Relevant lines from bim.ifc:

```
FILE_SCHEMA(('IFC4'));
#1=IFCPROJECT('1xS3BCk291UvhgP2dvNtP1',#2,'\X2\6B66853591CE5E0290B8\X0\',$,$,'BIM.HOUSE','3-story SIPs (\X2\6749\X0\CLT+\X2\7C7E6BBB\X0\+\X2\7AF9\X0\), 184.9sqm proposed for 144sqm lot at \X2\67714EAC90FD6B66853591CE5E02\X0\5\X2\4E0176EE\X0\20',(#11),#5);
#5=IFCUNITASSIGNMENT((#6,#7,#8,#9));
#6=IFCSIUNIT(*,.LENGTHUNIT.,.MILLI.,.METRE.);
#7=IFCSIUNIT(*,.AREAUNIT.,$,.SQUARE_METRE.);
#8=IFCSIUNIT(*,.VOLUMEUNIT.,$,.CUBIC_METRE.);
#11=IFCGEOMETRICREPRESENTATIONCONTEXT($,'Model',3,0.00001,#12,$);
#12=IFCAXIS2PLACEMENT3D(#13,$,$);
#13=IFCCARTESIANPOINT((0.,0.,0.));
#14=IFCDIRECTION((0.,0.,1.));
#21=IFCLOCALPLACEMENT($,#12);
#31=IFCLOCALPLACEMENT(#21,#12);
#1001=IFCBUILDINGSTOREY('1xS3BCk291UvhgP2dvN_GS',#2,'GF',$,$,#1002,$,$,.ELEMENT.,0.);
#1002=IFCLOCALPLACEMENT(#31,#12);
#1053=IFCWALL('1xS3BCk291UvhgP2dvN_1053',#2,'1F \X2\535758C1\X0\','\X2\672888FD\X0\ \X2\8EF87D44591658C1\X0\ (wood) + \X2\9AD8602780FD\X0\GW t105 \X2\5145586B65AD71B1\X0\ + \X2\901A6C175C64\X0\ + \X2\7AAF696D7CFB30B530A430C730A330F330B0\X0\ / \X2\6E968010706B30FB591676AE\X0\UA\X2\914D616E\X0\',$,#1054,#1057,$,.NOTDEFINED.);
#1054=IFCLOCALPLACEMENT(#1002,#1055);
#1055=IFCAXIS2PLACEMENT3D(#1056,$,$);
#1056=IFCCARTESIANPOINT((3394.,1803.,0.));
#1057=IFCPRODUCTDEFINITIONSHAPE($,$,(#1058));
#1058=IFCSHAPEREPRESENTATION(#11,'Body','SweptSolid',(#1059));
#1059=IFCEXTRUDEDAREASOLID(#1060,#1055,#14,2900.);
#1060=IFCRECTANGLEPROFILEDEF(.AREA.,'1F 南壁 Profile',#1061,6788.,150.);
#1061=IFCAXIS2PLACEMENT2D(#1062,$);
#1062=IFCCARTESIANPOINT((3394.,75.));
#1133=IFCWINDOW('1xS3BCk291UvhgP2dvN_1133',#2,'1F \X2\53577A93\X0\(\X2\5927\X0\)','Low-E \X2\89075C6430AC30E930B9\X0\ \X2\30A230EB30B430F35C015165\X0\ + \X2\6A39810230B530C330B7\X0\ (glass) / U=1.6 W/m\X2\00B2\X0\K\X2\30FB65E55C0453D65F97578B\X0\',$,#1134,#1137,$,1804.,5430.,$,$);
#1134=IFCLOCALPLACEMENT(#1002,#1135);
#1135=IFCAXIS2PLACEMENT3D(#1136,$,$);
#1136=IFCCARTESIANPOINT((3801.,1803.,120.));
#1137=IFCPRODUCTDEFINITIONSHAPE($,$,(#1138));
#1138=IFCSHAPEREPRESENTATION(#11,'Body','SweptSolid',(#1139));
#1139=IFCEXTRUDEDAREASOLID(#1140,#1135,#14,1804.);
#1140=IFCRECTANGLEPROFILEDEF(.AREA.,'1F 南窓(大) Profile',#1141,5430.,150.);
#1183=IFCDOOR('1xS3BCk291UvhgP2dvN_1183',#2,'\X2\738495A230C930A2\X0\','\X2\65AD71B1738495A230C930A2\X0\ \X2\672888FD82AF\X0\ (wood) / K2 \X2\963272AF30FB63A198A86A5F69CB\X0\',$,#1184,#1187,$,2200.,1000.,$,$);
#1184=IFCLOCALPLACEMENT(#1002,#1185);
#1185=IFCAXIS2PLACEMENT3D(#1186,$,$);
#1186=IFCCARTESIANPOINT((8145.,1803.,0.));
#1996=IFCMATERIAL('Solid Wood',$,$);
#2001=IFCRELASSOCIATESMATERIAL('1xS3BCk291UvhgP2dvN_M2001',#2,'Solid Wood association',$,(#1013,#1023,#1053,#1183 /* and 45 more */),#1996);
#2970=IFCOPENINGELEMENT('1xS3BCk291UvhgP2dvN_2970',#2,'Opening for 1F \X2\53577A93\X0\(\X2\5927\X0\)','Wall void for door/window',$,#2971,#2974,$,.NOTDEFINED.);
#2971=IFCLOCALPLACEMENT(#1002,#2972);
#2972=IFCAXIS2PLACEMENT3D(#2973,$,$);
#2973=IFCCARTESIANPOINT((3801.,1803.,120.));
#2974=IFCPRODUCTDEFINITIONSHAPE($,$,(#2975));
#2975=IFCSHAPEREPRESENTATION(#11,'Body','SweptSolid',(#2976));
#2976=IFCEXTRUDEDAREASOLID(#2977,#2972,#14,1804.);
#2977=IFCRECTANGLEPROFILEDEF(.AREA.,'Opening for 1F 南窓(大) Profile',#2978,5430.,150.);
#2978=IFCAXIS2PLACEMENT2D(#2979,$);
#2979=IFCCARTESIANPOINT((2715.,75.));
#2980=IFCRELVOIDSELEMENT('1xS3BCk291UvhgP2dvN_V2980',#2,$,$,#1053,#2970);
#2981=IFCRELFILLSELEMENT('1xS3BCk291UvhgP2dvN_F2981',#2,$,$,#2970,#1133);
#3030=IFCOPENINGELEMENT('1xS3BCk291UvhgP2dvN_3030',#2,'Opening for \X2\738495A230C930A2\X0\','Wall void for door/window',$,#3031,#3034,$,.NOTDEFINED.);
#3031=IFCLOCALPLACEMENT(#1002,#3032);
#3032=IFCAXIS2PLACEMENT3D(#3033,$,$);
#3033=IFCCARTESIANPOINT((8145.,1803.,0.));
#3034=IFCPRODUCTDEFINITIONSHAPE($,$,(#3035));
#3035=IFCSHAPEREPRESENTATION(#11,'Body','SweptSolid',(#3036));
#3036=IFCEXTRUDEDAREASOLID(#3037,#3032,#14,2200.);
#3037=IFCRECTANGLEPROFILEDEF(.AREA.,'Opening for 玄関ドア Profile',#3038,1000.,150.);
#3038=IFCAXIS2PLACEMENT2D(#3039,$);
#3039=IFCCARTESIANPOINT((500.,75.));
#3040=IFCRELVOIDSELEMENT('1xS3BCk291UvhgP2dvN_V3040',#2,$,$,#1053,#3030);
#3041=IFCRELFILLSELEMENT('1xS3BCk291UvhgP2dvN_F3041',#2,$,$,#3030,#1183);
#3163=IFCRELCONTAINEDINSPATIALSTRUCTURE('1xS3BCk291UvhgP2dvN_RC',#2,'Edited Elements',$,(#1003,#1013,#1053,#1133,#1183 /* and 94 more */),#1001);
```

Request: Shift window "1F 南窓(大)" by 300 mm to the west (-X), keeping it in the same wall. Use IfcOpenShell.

```python
import ifcopenshell
import ifcopenshell.api.geometry
import ifcopenshell.util.placement

model = ifcopenshell.open("bim.ifc")

window = model.by_guid("1xS3BCk291UvhgP2dvN_1133")
opening = window.FillsVoids[0].RelatingOpeningElement
wall = opening.VoidsElements[0].RelatingBuildingElement

wall_matrix = ifcopenshell.util.placement.get_local_placement(wall.ObjectPlacement)
shift = wall_matrix[:3, 0] * -300.0
before = ifcopenshell.util.placement.get_local_placement(window.ObjectPlacement)[:3, 3].copy()

# The window is not placed relative to its opening, so move both.
for product in (opening, window):
    matrix = ifcopenshell.util.placement.get_local_placement(product.ObjectPlacement)
    matrix[:3, 3] += shift
    ifcopenshell.api.geometry.edit_object_placement(model, product=product, matrix=matrix, is_si=False)

after = ifcopenshell.util.placement.get_local_placement(window.ObjectPlacement)[:3, 3]
print("window moved by", (after - before).round(3) + 0.0)

model.write("bim-out.ifc")
```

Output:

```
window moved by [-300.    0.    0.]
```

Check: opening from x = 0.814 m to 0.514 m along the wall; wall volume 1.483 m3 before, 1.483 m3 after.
